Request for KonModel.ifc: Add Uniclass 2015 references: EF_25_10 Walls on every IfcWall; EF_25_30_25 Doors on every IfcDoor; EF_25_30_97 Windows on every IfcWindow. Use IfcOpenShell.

First a look at what the model holds.

```python
import ifcopenshell

model = ifcopenshell.open("KonModel.ifc")
print(model.schema)
print("classifications:", [c.Name for c in model.by_type("IfcClassification")])
for ifc_class in ("IfcDoor", "IfcRoof", "IfcStair", "IfcWall", "IfcWindow"):
    print(ifc_class, len(model.by_type(ifc_class)))
```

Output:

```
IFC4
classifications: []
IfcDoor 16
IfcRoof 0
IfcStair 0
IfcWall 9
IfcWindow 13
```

```python
import ifcopenshell
import ifcopenshell.api.classification

model = ifcopenshell.open("KonModel.ifc")

system = ifcopenshell.api.classification.add_classification(model, classification="Uniclass 2015")

codes = {
    "IfcWall": ("EF_25_10", "Walls"),
    "IfcDoor": ("EF_25_30_25", "Doors"),
    "IfcWindow": ("EF_25_30_97", "Windows"),
}
for ifc_class, (code, name) in codes.items():
    products = model.by_type(ifc_class)
    ifcopenshell.api.classification.add_reference(
        model, products=products, classification=system, identification=code, name=name
    )
    print(code, len(products))

model.write("KonModel-out.ifc")
```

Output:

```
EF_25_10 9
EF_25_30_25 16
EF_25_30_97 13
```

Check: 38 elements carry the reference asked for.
